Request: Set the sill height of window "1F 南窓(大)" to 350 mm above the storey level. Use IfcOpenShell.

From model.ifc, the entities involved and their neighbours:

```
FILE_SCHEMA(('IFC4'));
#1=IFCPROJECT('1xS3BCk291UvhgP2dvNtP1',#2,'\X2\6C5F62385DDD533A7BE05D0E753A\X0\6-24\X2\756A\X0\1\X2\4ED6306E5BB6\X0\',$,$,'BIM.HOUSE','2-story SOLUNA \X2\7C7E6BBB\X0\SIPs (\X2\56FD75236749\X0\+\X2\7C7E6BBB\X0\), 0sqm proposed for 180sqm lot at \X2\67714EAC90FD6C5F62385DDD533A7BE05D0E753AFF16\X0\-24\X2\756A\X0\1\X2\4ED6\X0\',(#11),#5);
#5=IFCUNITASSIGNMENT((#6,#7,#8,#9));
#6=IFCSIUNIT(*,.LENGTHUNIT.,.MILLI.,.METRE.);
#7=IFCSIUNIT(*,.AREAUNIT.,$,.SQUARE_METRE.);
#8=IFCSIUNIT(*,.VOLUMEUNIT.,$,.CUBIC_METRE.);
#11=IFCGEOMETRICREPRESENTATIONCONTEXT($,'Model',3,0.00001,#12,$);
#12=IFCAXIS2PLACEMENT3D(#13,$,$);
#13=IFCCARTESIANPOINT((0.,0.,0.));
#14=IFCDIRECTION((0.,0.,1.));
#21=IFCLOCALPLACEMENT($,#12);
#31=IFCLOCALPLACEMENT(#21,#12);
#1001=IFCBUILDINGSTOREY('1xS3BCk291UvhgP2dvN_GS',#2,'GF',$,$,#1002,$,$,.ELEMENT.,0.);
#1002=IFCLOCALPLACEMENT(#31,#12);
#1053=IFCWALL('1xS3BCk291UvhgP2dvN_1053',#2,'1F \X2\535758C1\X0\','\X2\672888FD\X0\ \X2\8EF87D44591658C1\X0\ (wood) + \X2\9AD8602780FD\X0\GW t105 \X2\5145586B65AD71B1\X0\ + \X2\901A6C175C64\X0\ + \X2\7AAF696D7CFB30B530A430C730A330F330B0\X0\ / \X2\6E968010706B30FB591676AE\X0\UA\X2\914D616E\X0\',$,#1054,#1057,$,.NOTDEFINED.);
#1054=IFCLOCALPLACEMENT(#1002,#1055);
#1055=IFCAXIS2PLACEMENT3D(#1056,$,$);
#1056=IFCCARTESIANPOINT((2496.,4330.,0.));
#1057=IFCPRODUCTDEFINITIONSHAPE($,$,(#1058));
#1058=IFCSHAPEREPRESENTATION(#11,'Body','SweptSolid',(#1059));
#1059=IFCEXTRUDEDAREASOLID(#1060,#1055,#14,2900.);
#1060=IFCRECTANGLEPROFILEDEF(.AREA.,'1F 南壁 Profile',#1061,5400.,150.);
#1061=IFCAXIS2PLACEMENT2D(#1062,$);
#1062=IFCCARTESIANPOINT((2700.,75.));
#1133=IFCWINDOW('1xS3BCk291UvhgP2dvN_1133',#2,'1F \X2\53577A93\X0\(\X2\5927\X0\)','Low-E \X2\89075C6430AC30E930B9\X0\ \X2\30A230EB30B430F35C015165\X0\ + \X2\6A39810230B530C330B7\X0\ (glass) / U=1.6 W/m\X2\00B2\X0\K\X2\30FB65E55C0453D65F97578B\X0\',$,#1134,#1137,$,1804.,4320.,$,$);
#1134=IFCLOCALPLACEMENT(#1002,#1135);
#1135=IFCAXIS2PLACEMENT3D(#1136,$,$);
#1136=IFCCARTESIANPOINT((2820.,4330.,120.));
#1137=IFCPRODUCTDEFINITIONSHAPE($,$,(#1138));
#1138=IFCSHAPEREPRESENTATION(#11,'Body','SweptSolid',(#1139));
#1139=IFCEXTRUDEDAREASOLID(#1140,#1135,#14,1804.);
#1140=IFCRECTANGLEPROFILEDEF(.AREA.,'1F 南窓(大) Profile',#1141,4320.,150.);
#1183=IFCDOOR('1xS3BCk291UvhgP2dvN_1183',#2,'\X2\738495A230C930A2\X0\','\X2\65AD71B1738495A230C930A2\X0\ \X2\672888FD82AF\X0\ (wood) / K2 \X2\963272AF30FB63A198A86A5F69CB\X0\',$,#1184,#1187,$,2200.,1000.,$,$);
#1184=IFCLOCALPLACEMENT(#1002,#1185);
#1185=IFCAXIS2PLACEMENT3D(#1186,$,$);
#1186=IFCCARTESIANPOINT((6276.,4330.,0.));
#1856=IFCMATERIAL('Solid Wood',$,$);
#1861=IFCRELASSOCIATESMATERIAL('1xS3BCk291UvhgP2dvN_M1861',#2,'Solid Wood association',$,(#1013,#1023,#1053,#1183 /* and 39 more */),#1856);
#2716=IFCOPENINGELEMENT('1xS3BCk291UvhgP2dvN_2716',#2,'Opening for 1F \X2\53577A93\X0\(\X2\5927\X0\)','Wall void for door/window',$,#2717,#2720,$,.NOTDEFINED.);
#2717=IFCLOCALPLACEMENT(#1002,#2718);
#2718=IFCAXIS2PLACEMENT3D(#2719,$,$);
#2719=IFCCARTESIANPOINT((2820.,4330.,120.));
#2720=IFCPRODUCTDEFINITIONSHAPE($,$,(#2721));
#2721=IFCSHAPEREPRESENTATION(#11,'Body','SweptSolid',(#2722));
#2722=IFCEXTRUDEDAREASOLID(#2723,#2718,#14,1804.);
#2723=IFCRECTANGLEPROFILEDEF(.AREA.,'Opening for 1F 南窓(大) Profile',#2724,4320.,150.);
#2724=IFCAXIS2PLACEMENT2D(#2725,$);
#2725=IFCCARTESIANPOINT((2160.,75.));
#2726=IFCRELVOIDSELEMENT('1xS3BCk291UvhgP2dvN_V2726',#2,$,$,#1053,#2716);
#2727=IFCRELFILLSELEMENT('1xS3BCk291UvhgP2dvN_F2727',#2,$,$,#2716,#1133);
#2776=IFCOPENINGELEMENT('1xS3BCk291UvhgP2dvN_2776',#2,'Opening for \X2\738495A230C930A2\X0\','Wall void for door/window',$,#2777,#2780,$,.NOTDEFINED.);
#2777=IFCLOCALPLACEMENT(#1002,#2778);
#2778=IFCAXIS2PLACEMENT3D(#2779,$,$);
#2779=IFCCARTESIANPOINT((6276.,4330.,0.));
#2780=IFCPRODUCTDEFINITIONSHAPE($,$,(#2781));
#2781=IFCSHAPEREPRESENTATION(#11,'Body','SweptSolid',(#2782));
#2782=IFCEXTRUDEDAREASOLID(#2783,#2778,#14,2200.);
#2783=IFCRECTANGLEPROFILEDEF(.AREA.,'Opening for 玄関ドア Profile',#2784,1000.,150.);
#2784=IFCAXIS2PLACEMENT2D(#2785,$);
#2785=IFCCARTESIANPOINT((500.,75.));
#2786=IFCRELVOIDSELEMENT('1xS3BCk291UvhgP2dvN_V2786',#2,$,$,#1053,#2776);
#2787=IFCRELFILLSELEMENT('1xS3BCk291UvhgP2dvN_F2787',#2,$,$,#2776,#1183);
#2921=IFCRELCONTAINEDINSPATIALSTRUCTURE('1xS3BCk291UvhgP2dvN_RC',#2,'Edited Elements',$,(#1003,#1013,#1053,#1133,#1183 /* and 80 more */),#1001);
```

```python
import numpy as np
import ifcopenshell
import ifcopenshell.api.geometry
import ifcopenshell.geom
import ifcopenshell.util.element
import ifcopenshell.util.placement
import ifcopenshell.util.shape
import ifcopenshell.util.unit

model = ifcopenshell.open("model.ifc")
unit_scale = ifcopenshell.util.unit.calculate_unit_scale(model)

window = model.by_id(1133)
opening = window.FillsVoids[0].RelatingOpeningElement
storey = ifcopenshell.util.element.get_container(window, ifc_class="IfcBuildingStorey")
level = ifcopenshell.util.placement.get_local_placement(storey.ObjectPlacement)[2, 3]

# The opening's origin need not be at the sill, so measure its lowest point.
shape = ifcopenshell.geom.create_shape(ifcopenshell.geom.settings(), opening)
bottom = ifcopenshell.util.shape.get_shape_bottom_elevation(shape, shape.geometry) / unit_scale
dz = level + 0.35 / unit_scale - bottom

shift = np.array([0.0, 0.0, dz])
# The window is not placed relative to its opening, so move both.
for product in (opening, window):
    matrix = ifcopenshell.util.placement.get_local_placement(product.ObjectPlacement)
    matrix[:3, 3] += shift
    ifcopenshell.api.geometry.edit_object_placement(model, product=product, matrix=matrix, is_si=False)

print(f"moved by {dz * unit_scale:+.3f} m")

model.write("model_updated.ifc")
```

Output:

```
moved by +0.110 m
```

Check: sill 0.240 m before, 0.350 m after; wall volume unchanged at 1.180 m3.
